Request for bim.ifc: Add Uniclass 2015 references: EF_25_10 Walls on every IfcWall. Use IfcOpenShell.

First a look at what the model holds.

```python
import ifcopenshell

model = ifcopenshell.open("bim.ifc")
print(model.schema)
print("classifications:", [c.Name for c in model.by_type("IfcClassification")])
for ifc_class in ("IfcDoor", "IfcRoof", "IfcStair", "IfcWall", "IfcWindow"):
    print(ifc_class, len(model.by_type(ifc_class)))
```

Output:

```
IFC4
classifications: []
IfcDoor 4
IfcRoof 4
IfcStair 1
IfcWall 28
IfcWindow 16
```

```python
import ifcopenshell
import ifcopenshell.api.classification

model = ifcopenshell.open("bim.ifc")

system = ifcopenshell.api.classification.add_classification(model, classification="Uniclass 2015")

codes = {
    "IfcWall": ("EF_25_10", "Walls"),
}
for ifc_class, (code, name) in codes.items():
    products = model.by_type(ifc_class)
    ifcopenshell.api.classification.add_reference(
        model, products=products, classification=system, identification=code, name=name
    )
    print(code, len(products))

model.write("bim_edited.ifc")
```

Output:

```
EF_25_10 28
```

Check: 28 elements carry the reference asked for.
